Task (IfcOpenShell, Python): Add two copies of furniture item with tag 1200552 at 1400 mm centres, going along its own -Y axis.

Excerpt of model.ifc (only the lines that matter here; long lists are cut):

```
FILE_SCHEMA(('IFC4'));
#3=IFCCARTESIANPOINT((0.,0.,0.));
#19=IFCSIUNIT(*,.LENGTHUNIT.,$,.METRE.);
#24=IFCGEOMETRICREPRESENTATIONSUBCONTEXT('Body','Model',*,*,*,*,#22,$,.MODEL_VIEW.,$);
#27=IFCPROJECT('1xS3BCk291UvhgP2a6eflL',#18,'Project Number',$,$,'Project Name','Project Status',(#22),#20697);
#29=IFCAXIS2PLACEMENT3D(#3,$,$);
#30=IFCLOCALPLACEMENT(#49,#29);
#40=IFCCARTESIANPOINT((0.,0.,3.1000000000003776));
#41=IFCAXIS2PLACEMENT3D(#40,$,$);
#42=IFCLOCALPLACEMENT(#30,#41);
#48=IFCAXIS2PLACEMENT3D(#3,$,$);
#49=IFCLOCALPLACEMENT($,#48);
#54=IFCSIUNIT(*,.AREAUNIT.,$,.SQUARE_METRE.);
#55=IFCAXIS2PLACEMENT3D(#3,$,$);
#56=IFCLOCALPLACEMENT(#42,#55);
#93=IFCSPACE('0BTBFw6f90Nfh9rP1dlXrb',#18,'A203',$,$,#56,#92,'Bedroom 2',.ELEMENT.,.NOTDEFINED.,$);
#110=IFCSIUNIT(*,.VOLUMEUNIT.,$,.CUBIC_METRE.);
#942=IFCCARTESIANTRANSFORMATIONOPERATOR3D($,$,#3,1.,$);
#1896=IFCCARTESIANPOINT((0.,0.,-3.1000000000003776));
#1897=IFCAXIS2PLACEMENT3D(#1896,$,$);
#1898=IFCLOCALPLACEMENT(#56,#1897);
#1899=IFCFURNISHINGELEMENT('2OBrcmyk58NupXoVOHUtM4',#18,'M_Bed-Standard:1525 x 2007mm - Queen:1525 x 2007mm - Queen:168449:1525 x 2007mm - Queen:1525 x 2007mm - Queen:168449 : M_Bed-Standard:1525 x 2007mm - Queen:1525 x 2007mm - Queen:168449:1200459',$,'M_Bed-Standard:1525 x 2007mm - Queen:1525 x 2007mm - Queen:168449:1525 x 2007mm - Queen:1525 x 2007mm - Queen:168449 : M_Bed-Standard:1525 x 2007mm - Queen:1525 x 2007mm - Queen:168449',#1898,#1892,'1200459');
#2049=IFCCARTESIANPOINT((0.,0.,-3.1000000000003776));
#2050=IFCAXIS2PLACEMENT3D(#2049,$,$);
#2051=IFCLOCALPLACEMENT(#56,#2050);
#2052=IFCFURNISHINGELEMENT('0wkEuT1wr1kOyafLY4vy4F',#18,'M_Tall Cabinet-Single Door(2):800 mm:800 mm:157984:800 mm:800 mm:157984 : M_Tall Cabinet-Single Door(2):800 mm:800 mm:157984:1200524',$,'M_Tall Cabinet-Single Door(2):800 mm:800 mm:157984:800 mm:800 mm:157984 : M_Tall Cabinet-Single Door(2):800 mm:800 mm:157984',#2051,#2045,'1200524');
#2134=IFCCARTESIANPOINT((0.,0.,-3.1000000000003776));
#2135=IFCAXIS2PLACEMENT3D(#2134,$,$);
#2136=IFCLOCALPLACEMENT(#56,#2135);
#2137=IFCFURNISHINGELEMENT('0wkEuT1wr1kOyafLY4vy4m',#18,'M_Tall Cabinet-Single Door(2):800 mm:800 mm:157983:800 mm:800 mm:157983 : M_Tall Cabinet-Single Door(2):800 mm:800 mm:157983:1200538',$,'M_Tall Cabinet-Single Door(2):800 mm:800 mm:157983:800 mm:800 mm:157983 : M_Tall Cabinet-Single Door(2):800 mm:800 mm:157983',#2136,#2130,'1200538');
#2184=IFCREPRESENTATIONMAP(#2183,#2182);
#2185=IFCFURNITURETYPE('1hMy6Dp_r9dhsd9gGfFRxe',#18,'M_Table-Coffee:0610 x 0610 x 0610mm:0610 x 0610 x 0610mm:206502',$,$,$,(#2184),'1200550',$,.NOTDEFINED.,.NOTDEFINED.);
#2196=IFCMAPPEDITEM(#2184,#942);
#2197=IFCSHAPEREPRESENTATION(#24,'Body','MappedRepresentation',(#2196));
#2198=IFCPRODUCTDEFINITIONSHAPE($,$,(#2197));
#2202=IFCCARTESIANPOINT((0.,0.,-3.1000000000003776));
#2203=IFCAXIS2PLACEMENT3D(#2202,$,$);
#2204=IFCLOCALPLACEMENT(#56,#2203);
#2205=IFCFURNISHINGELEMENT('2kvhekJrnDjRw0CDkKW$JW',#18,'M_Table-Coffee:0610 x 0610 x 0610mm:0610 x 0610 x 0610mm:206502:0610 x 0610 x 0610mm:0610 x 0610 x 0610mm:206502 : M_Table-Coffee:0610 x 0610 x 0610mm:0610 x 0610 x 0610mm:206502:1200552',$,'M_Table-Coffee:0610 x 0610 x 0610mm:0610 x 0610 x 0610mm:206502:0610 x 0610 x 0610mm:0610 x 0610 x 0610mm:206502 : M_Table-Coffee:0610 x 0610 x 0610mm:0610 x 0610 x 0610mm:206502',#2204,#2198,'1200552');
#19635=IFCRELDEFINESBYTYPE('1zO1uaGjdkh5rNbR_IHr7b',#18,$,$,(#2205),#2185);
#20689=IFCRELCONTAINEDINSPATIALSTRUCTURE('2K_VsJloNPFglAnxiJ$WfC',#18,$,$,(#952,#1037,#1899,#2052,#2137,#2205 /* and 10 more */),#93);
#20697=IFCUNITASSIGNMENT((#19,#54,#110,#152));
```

```python
import ifcopenshell
import ifcopenshell.api.geometry
import ifcopenshell.api.root
import ifcopenshell.util.element
import ifcopenshell.util.placement

model = ifcopenshell.open("model.ifc")


def reuse_history(source, copy):
    """copy_class also copies each property set's owner history, people and application; keep the originals."""
    for rel in copy.IsDefinedBy:
        if rel.is_a("IfcRelDefinesByProperties") and (history := rel.RelatingPropertyDefinition.OwnerHistory):
            rel.RelatingPropertyDefinition.OwnerHistory = source.OwnerHistory
            ifcopenshell.util.element.remove_deep2(model, history)


source = model.by_guid("2kvhekJrnDjRw0CDkKW$JW")
base = ifcopenshell.util.placement.get_local_placement(source.ObjectPlacement)
step = -base[:3, 1] * 1.4

for i in range(1, 3):
    copy = ifcopenshell.api.root.copy_class(model, product=source)
    copy.Representation = ifcopenshell.util.element.copy_deep(
        model, source.Representation, exclude=["IfcGeometricRepresentationContext", "IfcRepresentationMap"]
    )
    copy.Name = "M_Table-Coffee:0610 x 0610 x 0610mm:0610 x 0610 x 0610mm:206502:0610 x 0610 x 0610mm:0610 x 0610 x 0610mm:206502 : M_Table-Coffee:0610 x 0610 x 0610mm:0610 x 0610 x 0610mm"
    copy.Tag = None
    reuse_history(source, copy)
    matrix = base.copy()
    matrix[:3, 3] += i * step
    print("added at", matrix[:3, 3].round(3) + 0.0)
    ifcopenshell.api.geometry.edit_object_placement(model, product=copy, matrix=matrix, is_si=False)

model.write("model_edited.ifc")
```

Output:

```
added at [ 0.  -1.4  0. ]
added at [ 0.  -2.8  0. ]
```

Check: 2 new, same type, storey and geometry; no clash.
